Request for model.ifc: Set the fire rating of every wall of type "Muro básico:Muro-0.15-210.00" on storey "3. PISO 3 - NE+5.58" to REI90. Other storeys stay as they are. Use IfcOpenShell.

First a look at what the model holds.

```python
import ifcopenshell
import ifcopenshell.util.element

model = ifcopenshell.open("model.ifc")
print(model.schema)
storey = next(s for s in model.by_type("IfcBuildingStorey") if s.Name == "3. PISO 3 - NE+5.58")
walls = [e for e in ifcopenshell.util.element.get_decomposition(storey) if e.is_a("IfcWall")]
seen = {}
for e in walls:
    element_type = ifcopenshell.util.element.get_type(e)
    key = (element_type.Name if element_type != e and element_type else None, ifcopenshell.util.element.get_pset(e, "Pset_WallCommon", "FireRating"))
    seen[key] = seen.get(key, 0) + 1
for (name, value), count in sorted(seen.items(), key=str):
    print(count, "x", name, "|", value)
```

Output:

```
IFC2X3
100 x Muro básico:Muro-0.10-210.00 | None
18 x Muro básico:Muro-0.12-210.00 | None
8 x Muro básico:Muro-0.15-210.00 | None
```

```python
import ifcopenshell
import ifcopenshell.api.pset
import ifcopenshell.util.element

model = ifcopenshell.open("model.ifc")

storey = next(s for s in model.by_type("IfcBuildingStorey") if s.Name == "3. PISO 3 - NE+5.58")
walls = [e for e in ifcopenshell.util.element.get_decomposition(storey) if e.is_a("IfcWall")]

count = 0
for e in walls:
    element_type = ifcopenshell.util.element.get_type(e)
    if element_type in (None, e) or element_type.Name != "Muro básico:Muro-0.15-210.00":
        continue
    # add_pset returns the element's existing set when there is one.
    pset = ifcopenshell.api.pset.add_pset(model, product=e, name="Pset_WallCommon")
    ifcopenshell.api.pset.edit_pset(model, pset=pset, properties={"FireRating": "REI90"})
    count += 1

print(count, "walls updated")

model.write("model_edited.ifc")
```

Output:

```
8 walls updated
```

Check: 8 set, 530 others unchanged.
